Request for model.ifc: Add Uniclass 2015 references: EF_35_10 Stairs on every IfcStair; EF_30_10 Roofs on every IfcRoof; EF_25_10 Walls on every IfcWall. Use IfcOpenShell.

First a look at what the model holds.

```python
import ifcopenshell

model = ifcopenshell.open("model.ifc")
print(model.schema)
print("classifications:", [c.Name for c in model.by_type("IfcClassification")])
for ifc_class in ("IfcDoor", "IfcRoof", "IfcStair", "IfcWall", "IfcWindow"):
    print(ifc_class, len(model.by_type(ifc_class)))
```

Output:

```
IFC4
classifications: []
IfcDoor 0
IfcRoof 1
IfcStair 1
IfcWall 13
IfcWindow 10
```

```python
import ifcopenshell
import ifcopenshell.api.classification

model = ifcopenshell.open("model.ifc")

system = ifcopenshell.api.classification.add_classification(model, classification="Uniclass 2015")

codes = {
    "IfcStair": ("EF_35_10", "Stairs"),
    "IfcRoof": ("EF_30_10", "Roofs"),
    "IfcWall": ("EF_25_10", "Walls"),
}
for ifc_class, (code, name) in codes.items():
    products = model.by_type(ifc_class)
    ifcopenshell.api.classification.add_reference(
        model, products=products, classification=system, identification=code, name=name
    )
    print(code, len(products))

model.write("model-out.ifc")
```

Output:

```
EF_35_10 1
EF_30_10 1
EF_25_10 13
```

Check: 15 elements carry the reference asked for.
